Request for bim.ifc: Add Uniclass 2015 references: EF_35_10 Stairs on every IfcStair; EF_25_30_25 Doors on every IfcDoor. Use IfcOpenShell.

First a look at what the model holds.

```python
import ifcopenshell

model = ifcopenshell.open("bim.ifc")
print(model.schema)
print("classifications:", [c.Name for c in model.by_type("IfcClassification")])
for ifc_class in ("IfcDoor", "IfcRoof", "IfcStair", "IfcWall", "IfcWindow"):
    print(ifc_class, len(model.by_type(ifc_class)))
```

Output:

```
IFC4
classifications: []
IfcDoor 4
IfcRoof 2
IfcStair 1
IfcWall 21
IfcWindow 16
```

```python
import ifcopenshell
import ifcopenshell.api.classification

model = ifcopenshell.open("bim.ifc")

system = ifcopenshell.api.classification.add_classification(model, classification="Uniclass 2015")

codes = {
    "IfcStair": ("EF_35_10", "Stairs"),
    "IfcDoor": ("EF_25_30_25", "Doors"),
}
for ifc_class, (code, name) in codes.items():
    products = model.by_type(ifc_class)
    ifcopenshell.api.classification.add_reference(
        model, products=products, classification=system, identification=code, name=name
    )
    print(code, len(products))

model.write("bim_rev.ifc")
```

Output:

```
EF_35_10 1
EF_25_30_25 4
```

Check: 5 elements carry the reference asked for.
